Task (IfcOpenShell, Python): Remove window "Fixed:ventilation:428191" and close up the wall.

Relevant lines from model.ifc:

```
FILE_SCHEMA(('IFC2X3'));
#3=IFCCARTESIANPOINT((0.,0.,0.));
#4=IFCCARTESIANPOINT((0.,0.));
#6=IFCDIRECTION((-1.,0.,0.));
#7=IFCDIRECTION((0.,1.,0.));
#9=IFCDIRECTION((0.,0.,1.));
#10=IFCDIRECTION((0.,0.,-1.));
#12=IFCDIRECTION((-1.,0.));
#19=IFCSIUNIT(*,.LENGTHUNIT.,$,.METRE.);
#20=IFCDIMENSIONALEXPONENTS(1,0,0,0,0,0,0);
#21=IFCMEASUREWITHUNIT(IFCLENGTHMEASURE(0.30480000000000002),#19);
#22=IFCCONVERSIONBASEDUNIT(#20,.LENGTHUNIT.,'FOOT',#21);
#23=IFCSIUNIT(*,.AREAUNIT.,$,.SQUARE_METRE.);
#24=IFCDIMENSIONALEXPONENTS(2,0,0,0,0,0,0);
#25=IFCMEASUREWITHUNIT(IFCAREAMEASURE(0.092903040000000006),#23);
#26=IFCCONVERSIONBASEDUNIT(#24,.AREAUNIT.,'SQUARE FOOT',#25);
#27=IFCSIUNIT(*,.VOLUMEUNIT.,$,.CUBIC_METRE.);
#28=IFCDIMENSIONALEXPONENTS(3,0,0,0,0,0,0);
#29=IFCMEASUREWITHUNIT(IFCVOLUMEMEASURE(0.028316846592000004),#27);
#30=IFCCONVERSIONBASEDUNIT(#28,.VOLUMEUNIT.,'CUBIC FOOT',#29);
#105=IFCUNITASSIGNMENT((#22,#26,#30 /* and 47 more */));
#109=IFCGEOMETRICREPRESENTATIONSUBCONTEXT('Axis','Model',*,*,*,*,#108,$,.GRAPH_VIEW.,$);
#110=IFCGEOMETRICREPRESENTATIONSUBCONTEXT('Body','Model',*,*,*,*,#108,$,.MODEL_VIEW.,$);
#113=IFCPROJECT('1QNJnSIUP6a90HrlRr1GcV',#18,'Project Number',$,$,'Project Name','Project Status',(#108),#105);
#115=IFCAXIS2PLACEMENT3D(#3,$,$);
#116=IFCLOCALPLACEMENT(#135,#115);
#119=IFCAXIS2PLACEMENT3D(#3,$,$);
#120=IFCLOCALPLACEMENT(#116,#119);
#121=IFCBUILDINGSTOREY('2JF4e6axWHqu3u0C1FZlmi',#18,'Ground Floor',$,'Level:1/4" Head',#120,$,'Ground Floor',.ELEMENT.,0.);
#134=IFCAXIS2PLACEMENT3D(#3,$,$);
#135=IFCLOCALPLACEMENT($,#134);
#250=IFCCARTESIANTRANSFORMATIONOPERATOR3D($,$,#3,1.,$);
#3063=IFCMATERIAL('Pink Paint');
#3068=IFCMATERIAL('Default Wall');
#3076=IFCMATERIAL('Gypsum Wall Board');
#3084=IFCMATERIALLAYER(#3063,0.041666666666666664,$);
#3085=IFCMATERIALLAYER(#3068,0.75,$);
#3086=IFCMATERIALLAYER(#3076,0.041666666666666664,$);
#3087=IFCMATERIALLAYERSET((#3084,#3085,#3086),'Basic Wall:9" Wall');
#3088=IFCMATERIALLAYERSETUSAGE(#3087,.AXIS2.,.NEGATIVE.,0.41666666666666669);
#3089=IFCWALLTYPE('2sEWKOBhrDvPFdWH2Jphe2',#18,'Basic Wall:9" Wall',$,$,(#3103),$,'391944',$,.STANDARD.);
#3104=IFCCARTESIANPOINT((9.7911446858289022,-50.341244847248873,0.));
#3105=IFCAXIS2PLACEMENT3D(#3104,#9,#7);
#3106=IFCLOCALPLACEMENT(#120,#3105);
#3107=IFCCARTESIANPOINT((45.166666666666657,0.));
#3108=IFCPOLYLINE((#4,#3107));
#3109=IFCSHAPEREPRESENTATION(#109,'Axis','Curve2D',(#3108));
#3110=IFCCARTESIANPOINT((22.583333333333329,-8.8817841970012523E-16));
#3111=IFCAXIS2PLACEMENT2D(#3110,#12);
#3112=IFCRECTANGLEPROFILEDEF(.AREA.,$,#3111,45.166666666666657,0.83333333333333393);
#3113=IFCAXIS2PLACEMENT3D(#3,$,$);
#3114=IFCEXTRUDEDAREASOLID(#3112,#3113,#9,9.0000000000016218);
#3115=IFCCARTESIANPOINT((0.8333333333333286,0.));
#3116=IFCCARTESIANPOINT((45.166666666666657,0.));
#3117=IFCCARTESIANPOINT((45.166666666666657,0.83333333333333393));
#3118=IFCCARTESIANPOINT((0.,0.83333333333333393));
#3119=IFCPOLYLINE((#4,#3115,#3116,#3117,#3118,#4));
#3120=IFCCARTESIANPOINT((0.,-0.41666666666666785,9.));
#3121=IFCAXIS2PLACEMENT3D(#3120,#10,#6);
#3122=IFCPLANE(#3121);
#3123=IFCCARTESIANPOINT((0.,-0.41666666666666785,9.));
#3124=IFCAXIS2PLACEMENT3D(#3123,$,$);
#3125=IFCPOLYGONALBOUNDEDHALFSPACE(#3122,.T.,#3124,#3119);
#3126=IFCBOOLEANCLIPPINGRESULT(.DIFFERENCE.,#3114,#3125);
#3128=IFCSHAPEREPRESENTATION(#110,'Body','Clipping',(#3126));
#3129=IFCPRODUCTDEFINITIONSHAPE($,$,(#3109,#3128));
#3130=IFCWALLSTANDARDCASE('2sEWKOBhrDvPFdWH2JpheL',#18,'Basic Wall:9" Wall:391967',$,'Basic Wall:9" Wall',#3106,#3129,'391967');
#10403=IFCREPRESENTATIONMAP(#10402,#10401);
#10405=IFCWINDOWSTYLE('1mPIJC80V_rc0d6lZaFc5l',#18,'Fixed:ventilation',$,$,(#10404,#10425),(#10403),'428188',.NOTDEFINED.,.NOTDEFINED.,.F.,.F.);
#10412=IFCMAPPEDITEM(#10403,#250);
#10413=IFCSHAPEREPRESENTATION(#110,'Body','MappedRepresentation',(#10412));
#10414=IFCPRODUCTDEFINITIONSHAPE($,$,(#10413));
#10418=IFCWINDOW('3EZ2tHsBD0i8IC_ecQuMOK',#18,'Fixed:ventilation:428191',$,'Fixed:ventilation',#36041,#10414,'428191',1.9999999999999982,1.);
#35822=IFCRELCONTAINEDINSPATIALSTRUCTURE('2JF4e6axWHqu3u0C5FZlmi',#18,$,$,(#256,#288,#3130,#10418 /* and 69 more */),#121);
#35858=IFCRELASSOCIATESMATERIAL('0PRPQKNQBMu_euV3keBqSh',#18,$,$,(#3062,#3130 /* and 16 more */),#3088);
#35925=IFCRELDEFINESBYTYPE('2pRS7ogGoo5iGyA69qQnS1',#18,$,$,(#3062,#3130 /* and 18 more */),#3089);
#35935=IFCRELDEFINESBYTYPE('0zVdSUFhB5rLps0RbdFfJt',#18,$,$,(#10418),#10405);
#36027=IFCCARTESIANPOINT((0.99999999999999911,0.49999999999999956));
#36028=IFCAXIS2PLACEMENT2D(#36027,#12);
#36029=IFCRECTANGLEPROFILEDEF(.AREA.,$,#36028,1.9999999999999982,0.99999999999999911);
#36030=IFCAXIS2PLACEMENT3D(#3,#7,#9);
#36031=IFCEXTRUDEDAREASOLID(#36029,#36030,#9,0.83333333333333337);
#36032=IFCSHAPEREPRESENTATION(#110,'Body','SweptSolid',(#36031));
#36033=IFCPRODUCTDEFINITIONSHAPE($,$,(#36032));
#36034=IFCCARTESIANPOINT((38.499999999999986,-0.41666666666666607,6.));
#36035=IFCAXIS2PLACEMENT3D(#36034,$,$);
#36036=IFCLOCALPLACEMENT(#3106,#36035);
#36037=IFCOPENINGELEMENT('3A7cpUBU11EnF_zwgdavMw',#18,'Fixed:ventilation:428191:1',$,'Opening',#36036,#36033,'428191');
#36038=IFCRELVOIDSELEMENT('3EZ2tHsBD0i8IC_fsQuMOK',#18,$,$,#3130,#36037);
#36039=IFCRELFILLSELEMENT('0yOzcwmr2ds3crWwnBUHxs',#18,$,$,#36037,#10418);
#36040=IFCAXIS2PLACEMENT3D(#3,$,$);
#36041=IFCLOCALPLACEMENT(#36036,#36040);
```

```python
import ifcopenshell
import ifcopenshell.api.feature
import ifcopenshell.api.root
import ifcopenshell.geom
import ifcopenshell.util.shape

model = ifcopenshell.open("model.ifc")
settings = ifcopenshell.geom.settings()


def volume(element):
    """Net volume in cubic metres, openings subtracted."""
    shape = ifcopenshell.geom.create_shape(settings, element)
    return ifcopenshell.util.shape.get_volume(shape.geometry)


window = model.by_guid("3EZ2tHsBD0i8IC_ecQuMOK")
opening = window.FillsVoids[0].RelatingOpeningElement
wall = opening.VoidsElements[0].RelatingBuildingElement
before = volume(wall)

ifcopenshell.api.root.remove_product(model, product=window)
ifcopenshell.api.feature.remove_feature(model, feature=opening)

after = volume(wall)

print(f"wall volume {before:.3f} -> {after:.3f} m3")

model.write("model_updated.ifc")
```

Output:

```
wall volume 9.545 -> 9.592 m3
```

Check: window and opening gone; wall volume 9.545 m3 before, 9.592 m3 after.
